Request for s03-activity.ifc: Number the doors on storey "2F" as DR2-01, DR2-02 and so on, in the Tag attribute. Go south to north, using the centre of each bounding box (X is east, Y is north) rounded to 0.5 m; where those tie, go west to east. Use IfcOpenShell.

First a look at what the model holds.

```python
import ifcopenshell
import ifcopenshell.util.element
import ifcopenshell.util.placement

model = ifcopenshell.open("s03-activity.ifc")
print(model.schema)
storey = next(s for s in model.by_type("IfcBuildingStorey") if s.Name == "2F")
doors = [e for e in ifcopenshell.util.element.get_decomposition(storey) if e.is_a("IfcDoor")]
for e in sorted(doors, key=lambda e: e.id()):
    origin = ifcopenshell.util.placement.get_local_placement(e.ObjectPlacement)[:3, 3]
    print(e.id(), e.Tag, e.Name, origin.round(2) + 0.0, sep=" | ")
```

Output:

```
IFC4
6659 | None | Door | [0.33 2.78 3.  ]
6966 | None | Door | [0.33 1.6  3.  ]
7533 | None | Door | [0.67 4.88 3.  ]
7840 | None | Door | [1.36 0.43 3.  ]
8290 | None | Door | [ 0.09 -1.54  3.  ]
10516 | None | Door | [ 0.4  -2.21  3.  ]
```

```python
import ifcopenshell
import ifcopenshell.geom
import ifcopenshell.util.element
import ifcopenshell.util.shape

model = ifcopenshell.open("s03-activity.ifc")
settings = ifcopenshell.geom.settings()
settings.set("use-world-coords", True)


def centre(element):
    shape = ifcopenshell.geom.create_shape(settings, element)
    return ifcopenshell.util.shape.get_bbox_centroid(shape.geometry)


storey = next(s for s in model.by_type("IfcBuildingStorey") if s.Name == "2F")
doors = [e for e in ifcopenshell.util.element.get_decomposition(storey) if e.is_a("IfcDoor")]

# Insertion points can sit at a corner or the storey origin, so sort by the geometry (in metres).
centres = {e: centre(e) for e in doors}
doors.sort(key=lambda e: (round(centres[e][1] / 0.5), centres[e][0]))

for i, e in enumerate(doors, start=1):
    number = f"DR2-{i:02d}"
    e.Tag = number
    print(e.id(), number)

model.write("s03-activity_rev.ifc")
```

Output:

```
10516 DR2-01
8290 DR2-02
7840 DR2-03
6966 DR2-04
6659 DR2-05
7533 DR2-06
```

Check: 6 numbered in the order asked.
